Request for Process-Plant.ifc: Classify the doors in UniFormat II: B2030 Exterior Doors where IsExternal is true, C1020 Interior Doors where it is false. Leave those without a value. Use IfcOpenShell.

First a look at what the model holds.

```python
import ifcopenshell
import ifcopenshell.util.element

model = ifcopenshell.open("Process-Plant.ifc")
print(model.schema)
print("classifications:", [c.Name for c in model.by_type("IfcClassification")])
values = [ifcopenshell.util.element.get_pset(e, "Pset_DoorCommon", "IsExternal") for e in model.by_type("IfcDoor")]
for value in (True, False, None):
    print("IsExternal", value, values.count(value))
```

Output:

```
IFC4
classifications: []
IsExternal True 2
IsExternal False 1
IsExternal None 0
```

```python
import ifcopenshell
import ifcopenshell.api.classification
import ifcopenshell.util.element

model = ifcopenshell.open("Process-Plant.ifc")

system = ifcopenshell.api.classification.add_classification(model, classification="UniFormat II")

doors = model.by_type("IfcDoor")
external = {e: ifcopenshell.util.element.get_pset(e, "Pset_DoorCommon", "IsExternal") for e in doors}
for flag, code, name in ((True, "B2030", "Exterior Doors"), (False, "C1020", "Interior Doors")):
    products = [e for e in doors if external[e] is flag]
    ifcopenshell.api.classification.add_reference(
        model, products=products, classification=system, identification=code, name=name
    )
    print(code, len(products))

model.write("Process-Plant_edited.ifc")
```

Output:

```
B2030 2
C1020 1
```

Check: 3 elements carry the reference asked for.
